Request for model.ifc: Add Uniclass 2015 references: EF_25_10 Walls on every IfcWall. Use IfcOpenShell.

First a look at what the model holds.

```python
import ifcopenshell

model = ifcopenshell.open("model.ifc")
print(model.schema)
print("classifications:", [c.Name for c in model.by_type("IfcClassification")])
for ifc_class in ("IfcDoor", "IfcRoof", "IfcStair", "IfcWall", "IfcWindow"):
    print(ifc_class, len(model.by_type(ifc_class)))
```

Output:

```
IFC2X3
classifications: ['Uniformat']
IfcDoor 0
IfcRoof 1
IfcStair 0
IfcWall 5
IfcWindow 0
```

```python
import ifcopenshell
import ifcopenshell.api.classification

model = ifcopenshell.open("model.ifc")

# IFC2X3 requires Source and Edition and has no link from the project to the system.
system = model.create_entity("IfcClassification", Source="NBS", Edition="2015", Name="Uniclass 2015")

codes = {
    "IfcWall": ("EF_25_10", "Walls"),
}
for ifc_class, (code, name) in codes.items():
    products = model.by_type(ifc_class)
    ifcopenshell.api.classification.add_reference(
        model, products=products, classification=system, identification=code, name=name
    )
    print(code, len(products))

model.write("model_updated.ifc")
```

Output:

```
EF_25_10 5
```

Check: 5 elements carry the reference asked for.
